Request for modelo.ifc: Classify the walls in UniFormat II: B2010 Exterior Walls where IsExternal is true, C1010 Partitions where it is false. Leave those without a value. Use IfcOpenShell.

First a look at what the model holds.

```python
import ifcopenshell
import ifcopenshell.util.element

model = ifcopenshell.open("modelo.ifc")
print(model.schema)
print("classifications:", [c.Name for c in model.by_type("IfcClassification")])
values = [ifcopenshell.util.element.get_pset(e, "Pset_WallCommon", "IsExternal") for e in model.by_type("IfcWall")]
for value in (True, False, None):
    print("IsExternal", value, values.count(value))
```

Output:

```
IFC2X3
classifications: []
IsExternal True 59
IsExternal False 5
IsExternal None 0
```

```python
import ifcopenshell
import ifcopenshell.api.classification
import ifcopenshell.util.element

model = ifcopenshell.open("modelo.ifc")

# IFC2X3 requires Source and Edition and has no link from the project to the system.
system = model.create_entity("IfcClassification", Source="ASTM", Edition="E1557", Name="UniFormat II")

walls = model.by_type("IfcWall")
external = {e: ifcopenshell.util.element.get_pset(e, "Pset_WallCommon", "IsExternal") for e in walls}
for flag, code, name in ((True, "B2010", "Exterior Walls"), (False, "C1010", "Partitions")):
    products = [e for e in walls if external[e] is flag]
    ifcopenshell.api.classification.add_reference(
        model, products=products, classification=system, identification=code, name=name
    )
    print(code, len(products))

model.write("modelo_v2.ifc")
```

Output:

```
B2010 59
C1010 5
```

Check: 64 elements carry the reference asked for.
